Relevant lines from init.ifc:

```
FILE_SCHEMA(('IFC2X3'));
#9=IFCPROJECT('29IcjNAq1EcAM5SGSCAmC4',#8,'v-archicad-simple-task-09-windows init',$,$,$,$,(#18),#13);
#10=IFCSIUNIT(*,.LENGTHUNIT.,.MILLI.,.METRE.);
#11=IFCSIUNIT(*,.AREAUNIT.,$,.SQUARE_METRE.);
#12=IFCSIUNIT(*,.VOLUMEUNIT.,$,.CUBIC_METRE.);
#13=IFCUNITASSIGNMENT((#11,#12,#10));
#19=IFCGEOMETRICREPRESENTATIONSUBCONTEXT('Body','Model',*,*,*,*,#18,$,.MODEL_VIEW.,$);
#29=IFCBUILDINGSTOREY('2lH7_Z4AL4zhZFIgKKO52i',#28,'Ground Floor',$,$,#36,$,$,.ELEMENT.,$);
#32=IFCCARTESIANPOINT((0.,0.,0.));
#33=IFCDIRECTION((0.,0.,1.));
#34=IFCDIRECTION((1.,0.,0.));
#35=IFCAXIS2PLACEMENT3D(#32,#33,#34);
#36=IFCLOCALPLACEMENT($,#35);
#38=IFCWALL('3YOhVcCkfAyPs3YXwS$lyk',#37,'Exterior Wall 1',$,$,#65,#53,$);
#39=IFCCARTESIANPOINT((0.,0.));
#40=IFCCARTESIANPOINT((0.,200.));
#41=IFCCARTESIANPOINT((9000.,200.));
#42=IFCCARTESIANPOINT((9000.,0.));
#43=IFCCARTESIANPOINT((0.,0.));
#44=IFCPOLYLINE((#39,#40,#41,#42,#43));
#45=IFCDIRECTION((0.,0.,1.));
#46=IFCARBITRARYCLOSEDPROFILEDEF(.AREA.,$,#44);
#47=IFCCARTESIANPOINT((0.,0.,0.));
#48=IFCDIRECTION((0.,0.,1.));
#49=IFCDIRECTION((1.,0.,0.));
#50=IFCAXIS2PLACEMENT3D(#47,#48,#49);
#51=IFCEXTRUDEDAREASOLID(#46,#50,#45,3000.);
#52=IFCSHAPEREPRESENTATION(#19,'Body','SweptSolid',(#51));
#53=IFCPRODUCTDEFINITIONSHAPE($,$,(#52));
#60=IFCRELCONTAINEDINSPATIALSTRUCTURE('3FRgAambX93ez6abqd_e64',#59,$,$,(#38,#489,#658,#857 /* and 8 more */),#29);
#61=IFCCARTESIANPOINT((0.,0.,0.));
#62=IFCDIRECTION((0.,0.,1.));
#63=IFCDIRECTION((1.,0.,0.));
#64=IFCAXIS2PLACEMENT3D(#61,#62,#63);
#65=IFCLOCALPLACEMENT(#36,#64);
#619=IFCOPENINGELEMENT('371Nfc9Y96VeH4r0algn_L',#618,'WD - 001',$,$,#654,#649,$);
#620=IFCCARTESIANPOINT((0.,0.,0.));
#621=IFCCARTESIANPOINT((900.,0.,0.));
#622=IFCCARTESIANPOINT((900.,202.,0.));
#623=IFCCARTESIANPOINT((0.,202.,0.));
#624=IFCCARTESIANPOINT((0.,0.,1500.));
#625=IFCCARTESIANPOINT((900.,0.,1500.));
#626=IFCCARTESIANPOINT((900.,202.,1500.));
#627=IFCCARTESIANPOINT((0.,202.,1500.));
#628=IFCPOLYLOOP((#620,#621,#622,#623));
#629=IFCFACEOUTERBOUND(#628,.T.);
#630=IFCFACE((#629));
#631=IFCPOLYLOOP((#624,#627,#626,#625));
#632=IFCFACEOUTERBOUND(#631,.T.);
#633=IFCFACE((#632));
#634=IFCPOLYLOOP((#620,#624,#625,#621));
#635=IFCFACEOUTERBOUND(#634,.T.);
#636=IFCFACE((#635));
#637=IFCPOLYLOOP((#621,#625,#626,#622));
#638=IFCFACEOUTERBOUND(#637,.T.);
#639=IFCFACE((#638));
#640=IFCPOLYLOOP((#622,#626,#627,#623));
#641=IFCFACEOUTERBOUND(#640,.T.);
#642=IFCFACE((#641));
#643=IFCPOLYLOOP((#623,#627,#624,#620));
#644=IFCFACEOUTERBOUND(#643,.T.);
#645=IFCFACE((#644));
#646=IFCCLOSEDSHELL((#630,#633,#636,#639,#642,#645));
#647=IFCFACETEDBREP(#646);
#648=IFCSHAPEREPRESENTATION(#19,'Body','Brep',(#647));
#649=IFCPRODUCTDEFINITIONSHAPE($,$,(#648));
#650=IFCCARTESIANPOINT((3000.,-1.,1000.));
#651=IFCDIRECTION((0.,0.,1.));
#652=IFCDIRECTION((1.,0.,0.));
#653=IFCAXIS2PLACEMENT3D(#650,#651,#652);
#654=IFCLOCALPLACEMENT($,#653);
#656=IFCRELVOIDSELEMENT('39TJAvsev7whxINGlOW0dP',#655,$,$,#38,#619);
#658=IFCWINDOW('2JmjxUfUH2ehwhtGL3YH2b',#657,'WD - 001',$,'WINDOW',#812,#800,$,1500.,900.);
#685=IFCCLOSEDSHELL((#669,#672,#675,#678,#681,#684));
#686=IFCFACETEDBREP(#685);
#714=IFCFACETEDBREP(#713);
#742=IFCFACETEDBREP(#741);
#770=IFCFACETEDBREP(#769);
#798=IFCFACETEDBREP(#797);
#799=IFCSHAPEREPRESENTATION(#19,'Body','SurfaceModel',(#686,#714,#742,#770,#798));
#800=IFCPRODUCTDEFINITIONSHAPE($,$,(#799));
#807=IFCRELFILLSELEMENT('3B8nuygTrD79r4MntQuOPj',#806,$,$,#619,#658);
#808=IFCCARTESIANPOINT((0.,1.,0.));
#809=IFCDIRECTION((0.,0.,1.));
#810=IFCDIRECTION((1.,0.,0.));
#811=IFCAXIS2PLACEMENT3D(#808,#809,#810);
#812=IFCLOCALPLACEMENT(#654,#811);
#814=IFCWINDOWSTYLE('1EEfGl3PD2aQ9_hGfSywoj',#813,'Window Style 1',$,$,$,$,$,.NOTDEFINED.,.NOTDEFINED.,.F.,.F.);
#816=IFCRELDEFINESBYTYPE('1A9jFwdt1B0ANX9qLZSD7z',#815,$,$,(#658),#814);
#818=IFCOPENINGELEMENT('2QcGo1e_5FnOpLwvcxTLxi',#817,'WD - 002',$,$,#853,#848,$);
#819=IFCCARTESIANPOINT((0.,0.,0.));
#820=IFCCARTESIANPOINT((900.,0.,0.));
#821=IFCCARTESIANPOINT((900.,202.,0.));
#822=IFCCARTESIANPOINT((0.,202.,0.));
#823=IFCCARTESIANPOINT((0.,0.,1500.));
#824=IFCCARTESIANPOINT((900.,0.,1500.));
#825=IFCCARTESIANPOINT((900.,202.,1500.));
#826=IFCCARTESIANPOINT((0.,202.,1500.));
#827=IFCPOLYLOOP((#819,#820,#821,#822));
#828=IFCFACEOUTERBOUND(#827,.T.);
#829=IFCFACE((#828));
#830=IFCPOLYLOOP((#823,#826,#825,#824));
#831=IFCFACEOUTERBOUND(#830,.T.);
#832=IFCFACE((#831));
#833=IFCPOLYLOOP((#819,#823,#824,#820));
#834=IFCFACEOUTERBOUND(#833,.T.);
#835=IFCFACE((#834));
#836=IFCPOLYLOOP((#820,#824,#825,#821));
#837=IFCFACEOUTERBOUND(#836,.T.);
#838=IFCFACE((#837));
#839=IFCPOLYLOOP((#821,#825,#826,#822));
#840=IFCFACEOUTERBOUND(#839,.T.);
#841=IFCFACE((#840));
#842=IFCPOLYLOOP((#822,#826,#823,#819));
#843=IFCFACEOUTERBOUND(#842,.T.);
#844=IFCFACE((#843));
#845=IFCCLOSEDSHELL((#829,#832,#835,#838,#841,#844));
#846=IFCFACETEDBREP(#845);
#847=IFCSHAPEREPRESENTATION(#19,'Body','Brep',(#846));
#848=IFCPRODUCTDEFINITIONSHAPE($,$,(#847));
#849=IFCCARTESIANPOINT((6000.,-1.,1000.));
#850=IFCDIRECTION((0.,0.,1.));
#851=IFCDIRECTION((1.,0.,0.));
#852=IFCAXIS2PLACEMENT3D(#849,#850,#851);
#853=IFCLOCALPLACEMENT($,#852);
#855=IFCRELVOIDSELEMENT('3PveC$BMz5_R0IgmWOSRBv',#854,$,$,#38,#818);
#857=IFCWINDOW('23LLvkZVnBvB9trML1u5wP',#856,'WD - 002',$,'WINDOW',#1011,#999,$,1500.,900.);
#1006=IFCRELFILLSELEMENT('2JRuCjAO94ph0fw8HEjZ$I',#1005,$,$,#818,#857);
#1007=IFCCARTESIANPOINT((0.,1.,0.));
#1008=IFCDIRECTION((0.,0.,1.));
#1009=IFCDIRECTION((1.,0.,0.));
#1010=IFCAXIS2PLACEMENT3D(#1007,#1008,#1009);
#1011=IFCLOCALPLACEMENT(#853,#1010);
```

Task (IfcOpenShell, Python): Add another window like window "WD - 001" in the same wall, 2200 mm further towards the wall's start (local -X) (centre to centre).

```python
import ifcopenshell
import ifcopenshell.api.feature
import ifcopenshell.api.geometry
import ifcopenshell.api.root
import ifcopenshell.geom
import ifcopenshell.util.element
import ifcopenshell.util.placement
import ifcopenshell.util.shape

model = ifcopenshell.open("init.ifc")
settings = ifcopenshell.geom.settings()


def volume(element):
    """Net volume in cubic metres, openings subtracted."""
    shape = ifcopenshell.geom.create_shape(settings, element)
    return ifcopenshell.util.shape.get_volume(shape.geometry)


window = model.by_id(658)
opening = window.FillsVoids[0].RelatingOpeningElement
wall = opening.VoidsElements[0].RelatingBuildingElement
before = volume(wall)
shift = ifcopenshell.util.placement.get_local_placement(wall.ObjectPlacement)[:3, 0] * -2200.0

# copy_class copies the void relationship, type, container and properties, but no geometry.
new_opening = ifcopenshell.api.root.copy_class(model, product=opening)
new_opening.Representation = ifcopenshell.util.element.copy_deep(
    model, opening.Representation, exclude=["IfcGeometricRepresentationContext", "IfcRepresentationMap"]
)
new_window = ifcopenshell.api.root.copy_class(model, product=window)
new_window.Representation = ifcopenshell.util.element.copy_deep(
    model, window.Representation, exclude=["IfcGeometricRepresentationContext", "IfcRepresentationMap"]
)
fills = ifcopenshell.api.feature.add_filling(model, opening=new_opening, element=new_window)
fills.OwnerHistory = new_window.OwnerHistory  # required in IFC2X3

for old, new in ((opening, new_opening), (window, new_window)):
    matrix = ifcopenshell.util.placement.get_local_placement(old.ObjectPlacement)
    matrix[:3, 3] += shift
    ifcopenshell.api.geometry.edit_object_placement(model, product=new, matrix=matrix, is_si=False)

after = volume(wall)

print(f"wall volume {before:.3f} -> {after:.3f} m3")

model.write("init_edited.ifc")
```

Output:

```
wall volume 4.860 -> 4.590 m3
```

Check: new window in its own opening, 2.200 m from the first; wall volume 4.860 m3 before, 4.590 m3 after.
